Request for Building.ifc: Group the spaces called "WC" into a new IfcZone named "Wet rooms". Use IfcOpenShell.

First a look at what the model holds.

```python
import ifcopenshell

model = ifcopenshell.open("Building.ifc")
print(model.schema)
seen = {}
for space in model.by_type("IfcSpace"):
    seen[space.LongName] = seen.get(space.LongName, 0) + 1
for name, count in sorted(seen.items(), key=str):
    print(count, "x", name)
print("zones:", [z.Name for z in model.by_type("IfcZone")][:20])
```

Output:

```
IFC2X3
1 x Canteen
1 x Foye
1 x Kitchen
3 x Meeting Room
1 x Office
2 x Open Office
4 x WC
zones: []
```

```python
import ifcopenshell
import ifcopenshell.api.group
import ifcopenshell.api.root

model = ifcopenshell.open("Building.ifc")

names = {"WC"}
spaces = [s for s in model.by_type("IfcSpace") if s.LongName in names]

zone = ifcopenshell.api.root.create_entity(model, ifc_class="IfcZone", name="Wet rooms")
ifcopenshell.api.group.assign_group(model, products=spaces, group=zone)
print(len(spaces), "spaces in", zone.Name)

model.write("Building_updated.ifc")
```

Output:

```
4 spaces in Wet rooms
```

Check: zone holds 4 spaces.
